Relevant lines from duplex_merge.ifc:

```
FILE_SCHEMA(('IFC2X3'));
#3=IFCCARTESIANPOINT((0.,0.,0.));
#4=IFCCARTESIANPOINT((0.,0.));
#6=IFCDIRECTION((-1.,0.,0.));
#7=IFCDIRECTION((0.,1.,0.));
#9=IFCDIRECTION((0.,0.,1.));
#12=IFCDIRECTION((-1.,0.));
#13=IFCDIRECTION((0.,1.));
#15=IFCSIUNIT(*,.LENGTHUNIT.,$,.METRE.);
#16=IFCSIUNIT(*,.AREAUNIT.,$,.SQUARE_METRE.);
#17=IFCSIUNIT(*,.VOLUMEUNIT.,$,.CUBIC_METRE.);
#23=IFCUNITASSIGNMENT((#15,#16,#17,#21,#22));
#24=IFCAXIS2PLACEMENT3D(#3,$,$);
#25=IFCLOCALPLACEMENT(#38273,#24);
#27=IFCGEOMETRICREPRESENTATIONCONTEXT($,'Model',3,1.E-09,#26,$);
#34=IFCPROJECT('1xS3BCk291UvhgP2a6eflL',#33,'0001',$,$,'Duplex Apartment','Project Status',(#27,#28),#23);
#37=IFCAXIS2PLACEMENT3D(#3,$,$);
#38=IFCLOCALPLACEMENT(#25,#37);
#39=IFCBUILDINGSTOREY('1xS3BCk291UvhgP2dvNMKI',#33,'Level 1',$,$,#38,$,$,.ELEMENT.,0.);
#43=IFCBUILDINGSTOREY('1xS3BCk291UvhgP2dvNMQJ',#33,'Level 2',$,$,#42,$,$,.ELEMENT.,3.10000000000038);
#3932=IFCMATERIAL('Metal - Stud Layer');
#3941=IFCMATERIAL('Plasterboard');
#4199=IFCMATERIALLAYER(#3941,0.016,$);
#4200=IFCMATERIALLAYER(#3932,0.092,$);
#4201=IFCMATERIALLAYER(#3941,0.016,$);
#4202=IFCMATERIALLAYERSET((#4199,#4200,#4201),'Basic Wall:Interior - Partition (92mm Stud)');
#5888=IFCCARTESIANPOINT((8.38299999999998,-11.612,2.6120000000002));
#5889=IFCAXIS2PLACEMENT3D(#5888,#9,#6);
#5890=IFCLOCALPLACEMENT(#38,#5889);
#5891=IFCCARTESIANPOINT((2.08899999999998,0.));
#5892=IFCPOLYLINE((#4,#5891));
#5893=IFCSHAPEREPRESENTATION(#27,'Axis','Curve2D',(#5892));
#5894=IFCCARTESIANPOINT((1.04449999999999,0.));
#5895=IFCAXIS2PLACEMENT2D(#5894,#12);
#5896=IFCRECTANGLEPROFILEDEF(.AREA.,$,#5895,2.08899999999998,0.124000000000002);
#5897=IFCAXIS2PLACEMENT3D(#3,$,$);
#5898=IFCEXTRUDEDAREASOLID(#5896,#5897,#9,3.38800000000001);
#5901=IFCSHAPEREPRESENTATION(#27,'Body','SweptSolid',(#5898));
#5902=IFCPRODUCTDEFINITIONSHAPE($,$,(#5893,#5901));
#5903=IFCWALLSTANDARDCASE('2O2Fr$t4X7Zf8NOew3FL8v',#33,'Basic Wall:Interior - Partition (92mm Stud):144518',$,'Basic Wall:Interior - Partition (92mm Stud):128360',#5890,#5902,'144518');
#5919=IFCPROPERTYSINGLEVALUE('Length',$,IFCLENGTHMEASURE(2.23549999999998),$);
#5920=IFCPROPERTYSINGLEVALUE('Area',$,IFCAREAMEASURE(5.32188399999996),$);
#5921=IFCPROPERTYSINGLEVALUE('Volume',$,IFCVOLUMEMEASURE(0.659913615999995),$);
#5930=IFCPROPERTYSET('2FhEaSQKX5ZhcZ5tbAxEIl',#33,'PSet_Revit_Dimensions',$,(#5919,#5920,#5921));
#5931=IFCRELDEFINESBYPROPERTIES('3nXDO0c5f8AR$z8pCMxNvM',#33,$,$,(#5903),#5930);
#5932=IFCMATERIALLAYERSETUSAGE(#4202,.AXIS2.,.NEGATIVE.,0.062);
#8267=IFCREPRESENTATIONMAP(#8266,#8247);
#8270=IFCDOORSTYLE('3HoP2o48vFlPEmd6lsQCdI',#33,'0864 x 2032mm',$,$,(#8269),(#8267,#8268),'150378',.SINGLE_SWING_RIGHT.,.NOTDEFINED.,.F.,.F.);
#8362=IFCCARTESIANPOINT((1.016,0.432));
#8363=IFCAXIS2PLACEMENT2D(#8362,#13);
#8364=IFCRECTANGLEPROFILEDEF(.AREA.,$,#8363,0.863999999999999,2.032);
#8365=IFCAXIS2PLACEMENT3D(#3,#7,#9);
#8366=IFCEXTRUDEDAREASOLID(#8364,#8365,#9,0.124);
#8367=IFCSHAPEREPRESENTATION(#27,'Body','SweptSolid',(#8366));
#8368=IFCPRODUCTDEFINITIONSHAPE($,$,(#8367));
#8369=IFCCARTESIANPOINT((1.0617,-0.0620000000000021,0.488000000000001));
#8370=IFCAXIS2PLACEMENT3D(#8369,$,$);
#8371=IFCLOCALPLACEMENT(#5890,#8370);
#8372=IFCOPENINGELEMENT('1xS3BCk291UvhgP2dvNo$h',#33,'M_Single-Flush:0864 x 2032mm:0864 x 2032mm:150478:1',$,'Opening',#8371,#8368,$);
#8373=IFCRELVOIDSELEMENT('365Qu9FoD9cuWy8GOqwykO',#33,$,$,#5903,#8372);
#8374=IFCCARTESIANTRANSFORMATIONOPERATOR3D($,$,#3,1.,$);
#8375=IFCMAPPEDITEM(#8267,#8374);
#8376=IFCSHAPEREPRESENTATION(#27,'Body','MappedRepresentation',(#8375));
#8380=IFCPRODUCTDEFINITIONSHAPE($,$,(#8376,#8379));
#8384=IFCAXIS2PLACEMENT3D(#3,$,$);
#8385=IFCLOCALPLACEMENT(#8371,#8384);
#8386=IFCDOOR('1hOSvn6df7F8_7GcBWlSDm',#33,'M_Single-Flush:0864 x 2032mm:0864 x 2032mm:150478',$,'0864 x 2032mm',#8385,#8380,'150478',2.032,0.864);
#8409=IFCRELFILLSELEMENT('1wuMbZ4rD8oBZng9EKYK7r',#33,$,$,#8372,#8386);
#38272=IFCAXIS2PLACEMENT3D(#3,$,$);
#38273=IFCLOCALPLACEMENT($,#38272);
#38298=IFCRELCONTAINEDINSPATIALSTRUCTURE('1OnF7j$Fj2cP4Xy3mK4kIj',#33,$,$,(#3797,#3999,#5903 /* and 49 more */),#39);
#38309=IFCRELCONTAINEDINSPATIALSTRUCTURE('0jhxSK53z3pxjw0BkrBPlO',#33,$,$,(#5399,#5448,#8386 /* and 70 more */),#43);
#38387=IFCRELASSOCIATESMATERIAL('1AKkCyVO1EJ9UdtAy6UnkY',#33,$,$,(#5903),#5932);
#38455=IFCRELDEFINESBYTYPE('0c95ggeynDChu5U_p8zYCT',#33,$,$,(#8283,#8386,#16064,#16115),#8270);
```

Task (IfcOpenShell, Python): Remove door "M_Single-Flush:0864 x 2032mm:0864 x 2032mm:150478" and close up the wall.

```python
import ifcopenshell
import ifcopenshell.api.feature
import ifcopenshell.api.pset
import ifcopenshell.api.root
import ifcopenshell.geom
import ifcopenshell.util.element
import ifcopenshell.util.shape
import ifcopenshell.util.unit

model = ifcopenshell.open("duplex_merge.ifc")
area_scale = ifcopenshell.util.unit.calculate_unit_scale(model, "AREAUNIT")
volume_scale = ifcopenshell.util.unit.calculate_unit_scale(model, "VOLUMEUNIT")
settings = ifcopenshell.geom.settings()


def volume(element):
    """Net volume in cubic metres, openings subtracted."""
    shape = ifcopenshell.geom.create_shape(settings, element)
    return ifcopenshell.util.shape.get_volume(shape.geometry)


door = model.by_guid("1hOSvn6df7F8_7GcBWlSDm")
opening = door.FillsVoids[0].RelatingOpeningElement
wall = opening.VoidsElements[0].RelatingBuildingElement
before = volume(wall)

ifcopenshell.api.root.remove_product(model, product=door)
ifcopenshell.api.feature.remove_feature(model, feature=opening)

after = volume(wall)
thickness = 0.124  # wall thickness in metres

# Update the wall's stored quantities.
pset = model.by_id(ifcopenshell.util.element.get_pset(wall, "PSet_Revit_Dimensions", should_inherit=False)["id"])
ifcopenshell.api.pset.edit_pset(model, pset=pset, properties={
    "Area": model.create_entity("IfcAreaMeasure", after / thickness / area_scale),
    "Volume": model.create_entity("IfcVolumeMeasure", after / volume_scale),
})

print(f"wall volume {before:.3f} -> {after:.3f} m3")

model.write("duplex_merge_updated.ifc")
```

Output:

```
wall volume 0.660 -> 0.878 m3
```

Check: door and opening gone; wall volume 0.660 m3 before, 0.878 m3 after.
